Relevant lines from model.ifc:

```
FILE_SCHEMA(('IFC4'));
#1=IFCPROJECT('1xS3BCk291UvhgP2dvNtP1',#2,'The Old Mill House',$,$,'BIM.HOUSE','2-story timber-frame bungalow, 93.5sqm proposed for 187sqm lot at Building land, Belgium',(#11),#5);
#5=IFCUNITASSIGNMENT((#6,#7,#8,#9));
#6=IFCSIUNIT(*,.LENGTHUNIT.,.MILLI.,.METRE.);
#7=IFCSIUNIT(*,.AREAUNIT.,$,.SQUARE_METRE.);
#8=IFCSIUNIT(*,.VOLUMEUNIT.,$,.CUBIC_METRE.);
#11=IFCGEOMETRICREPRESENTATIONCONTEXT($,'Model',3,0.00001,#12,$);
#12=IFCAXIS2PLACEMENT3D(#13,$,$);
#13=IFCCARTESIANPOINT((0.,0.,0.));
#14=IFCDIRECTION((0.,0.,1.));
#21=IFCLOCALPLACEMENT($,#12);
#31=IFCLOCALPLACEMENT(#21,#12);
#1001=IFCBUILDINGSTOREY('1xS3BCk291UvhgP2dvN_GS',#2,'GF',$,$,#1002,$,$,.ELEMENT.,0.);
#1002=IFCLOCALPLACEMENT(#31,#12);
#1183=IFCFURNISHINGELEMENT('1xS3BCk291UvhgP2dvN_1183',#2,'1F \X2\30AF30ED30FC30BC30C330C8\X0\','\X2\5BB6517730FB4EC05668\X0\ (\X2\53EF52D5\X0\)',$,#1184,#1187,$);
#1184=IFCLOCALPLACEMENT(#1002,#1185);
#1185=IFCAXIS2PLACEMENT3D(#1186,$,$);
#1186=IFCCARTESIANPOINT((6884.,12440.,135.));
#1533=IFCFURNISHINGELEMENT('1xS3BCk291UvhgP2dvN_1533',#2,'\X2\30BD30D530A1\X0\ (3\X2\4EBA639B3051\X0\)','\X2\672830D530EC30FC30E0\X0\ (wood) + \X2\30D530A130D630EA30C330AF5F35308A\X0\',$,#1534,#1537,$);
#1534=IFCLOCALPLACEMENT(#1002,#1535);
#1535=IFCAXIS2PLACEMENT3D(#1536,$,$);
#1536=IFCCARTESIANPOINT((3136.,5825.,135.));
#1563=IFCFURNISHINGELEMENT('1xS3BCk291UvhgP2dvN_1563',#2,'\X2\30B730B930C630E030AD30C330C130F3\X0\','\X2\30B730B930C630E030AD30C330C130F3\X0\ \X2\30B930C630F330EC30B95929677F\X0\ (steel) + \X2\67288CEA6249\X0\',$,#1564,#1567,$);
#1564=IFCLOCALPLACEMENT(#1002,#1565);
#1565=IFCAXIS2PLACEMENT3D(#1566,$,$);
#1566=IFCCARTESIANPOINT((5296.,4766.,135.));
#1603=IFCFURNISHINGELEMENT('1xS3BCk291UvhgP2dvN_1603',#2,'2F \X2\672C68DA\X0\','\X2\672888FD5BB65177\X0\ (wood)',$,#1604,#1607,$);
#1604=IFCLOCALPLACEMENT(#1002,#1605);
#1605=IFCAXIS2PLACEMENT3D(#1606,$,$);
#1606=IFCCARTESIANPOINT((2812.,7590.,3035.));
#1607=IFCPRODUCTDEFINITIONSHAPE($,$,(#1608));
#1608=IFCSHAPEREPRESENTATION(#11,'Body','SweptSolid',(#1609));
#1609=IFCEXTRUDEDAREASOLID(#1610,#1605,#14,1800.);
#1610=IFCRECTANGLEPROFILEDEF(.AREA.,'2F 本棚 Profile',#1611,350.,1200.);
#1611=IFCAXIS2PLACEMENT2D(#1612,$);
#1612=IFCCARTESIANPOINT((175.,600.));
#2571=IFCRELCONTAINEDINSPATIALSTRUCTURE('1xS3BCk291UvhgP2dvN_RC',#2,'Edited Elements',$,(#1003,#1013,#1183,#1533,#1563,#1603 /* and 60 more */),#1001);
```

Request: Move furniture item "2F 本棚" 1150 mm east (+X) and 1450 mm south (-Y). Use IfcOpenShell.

```python
import ifcopenshell
import ifcopenshell.api.geometry
import ifcopenshell.util.placement
import ifcopenshell.util.unit

model = ifcopenshell.open("model.ifc")
unit_scale = ifcopenshell.util.unit.calculate_unit_scale(model)

item = model.by_guid("1xS3BCk291UvhgP2dvN_1603")
matrix = ifcopenshell.util.placement.get_local_placement(item.ObjectPlacement)
matrix[0, 3] += 1.15 / unit_scale
matrix[1, 3] -= 1.45 / unit_scale
ifcopenshell.api.geometry.edit_object_placement(model, product=item, matrix=matrix, is_si=False)

print(ifcopenshell.util.placement.get_local_placement(item.ObjectPlacement).round(3) + 0.0)

model.write("model_v2.ifc")
```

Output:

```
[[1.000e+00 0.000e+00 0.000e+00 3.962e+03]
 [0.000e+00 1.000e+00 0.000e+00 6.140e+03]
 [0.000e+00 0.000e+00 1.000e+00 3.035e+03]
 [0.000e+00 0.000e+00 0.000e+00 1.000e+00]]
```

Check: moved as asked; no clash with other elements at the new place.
